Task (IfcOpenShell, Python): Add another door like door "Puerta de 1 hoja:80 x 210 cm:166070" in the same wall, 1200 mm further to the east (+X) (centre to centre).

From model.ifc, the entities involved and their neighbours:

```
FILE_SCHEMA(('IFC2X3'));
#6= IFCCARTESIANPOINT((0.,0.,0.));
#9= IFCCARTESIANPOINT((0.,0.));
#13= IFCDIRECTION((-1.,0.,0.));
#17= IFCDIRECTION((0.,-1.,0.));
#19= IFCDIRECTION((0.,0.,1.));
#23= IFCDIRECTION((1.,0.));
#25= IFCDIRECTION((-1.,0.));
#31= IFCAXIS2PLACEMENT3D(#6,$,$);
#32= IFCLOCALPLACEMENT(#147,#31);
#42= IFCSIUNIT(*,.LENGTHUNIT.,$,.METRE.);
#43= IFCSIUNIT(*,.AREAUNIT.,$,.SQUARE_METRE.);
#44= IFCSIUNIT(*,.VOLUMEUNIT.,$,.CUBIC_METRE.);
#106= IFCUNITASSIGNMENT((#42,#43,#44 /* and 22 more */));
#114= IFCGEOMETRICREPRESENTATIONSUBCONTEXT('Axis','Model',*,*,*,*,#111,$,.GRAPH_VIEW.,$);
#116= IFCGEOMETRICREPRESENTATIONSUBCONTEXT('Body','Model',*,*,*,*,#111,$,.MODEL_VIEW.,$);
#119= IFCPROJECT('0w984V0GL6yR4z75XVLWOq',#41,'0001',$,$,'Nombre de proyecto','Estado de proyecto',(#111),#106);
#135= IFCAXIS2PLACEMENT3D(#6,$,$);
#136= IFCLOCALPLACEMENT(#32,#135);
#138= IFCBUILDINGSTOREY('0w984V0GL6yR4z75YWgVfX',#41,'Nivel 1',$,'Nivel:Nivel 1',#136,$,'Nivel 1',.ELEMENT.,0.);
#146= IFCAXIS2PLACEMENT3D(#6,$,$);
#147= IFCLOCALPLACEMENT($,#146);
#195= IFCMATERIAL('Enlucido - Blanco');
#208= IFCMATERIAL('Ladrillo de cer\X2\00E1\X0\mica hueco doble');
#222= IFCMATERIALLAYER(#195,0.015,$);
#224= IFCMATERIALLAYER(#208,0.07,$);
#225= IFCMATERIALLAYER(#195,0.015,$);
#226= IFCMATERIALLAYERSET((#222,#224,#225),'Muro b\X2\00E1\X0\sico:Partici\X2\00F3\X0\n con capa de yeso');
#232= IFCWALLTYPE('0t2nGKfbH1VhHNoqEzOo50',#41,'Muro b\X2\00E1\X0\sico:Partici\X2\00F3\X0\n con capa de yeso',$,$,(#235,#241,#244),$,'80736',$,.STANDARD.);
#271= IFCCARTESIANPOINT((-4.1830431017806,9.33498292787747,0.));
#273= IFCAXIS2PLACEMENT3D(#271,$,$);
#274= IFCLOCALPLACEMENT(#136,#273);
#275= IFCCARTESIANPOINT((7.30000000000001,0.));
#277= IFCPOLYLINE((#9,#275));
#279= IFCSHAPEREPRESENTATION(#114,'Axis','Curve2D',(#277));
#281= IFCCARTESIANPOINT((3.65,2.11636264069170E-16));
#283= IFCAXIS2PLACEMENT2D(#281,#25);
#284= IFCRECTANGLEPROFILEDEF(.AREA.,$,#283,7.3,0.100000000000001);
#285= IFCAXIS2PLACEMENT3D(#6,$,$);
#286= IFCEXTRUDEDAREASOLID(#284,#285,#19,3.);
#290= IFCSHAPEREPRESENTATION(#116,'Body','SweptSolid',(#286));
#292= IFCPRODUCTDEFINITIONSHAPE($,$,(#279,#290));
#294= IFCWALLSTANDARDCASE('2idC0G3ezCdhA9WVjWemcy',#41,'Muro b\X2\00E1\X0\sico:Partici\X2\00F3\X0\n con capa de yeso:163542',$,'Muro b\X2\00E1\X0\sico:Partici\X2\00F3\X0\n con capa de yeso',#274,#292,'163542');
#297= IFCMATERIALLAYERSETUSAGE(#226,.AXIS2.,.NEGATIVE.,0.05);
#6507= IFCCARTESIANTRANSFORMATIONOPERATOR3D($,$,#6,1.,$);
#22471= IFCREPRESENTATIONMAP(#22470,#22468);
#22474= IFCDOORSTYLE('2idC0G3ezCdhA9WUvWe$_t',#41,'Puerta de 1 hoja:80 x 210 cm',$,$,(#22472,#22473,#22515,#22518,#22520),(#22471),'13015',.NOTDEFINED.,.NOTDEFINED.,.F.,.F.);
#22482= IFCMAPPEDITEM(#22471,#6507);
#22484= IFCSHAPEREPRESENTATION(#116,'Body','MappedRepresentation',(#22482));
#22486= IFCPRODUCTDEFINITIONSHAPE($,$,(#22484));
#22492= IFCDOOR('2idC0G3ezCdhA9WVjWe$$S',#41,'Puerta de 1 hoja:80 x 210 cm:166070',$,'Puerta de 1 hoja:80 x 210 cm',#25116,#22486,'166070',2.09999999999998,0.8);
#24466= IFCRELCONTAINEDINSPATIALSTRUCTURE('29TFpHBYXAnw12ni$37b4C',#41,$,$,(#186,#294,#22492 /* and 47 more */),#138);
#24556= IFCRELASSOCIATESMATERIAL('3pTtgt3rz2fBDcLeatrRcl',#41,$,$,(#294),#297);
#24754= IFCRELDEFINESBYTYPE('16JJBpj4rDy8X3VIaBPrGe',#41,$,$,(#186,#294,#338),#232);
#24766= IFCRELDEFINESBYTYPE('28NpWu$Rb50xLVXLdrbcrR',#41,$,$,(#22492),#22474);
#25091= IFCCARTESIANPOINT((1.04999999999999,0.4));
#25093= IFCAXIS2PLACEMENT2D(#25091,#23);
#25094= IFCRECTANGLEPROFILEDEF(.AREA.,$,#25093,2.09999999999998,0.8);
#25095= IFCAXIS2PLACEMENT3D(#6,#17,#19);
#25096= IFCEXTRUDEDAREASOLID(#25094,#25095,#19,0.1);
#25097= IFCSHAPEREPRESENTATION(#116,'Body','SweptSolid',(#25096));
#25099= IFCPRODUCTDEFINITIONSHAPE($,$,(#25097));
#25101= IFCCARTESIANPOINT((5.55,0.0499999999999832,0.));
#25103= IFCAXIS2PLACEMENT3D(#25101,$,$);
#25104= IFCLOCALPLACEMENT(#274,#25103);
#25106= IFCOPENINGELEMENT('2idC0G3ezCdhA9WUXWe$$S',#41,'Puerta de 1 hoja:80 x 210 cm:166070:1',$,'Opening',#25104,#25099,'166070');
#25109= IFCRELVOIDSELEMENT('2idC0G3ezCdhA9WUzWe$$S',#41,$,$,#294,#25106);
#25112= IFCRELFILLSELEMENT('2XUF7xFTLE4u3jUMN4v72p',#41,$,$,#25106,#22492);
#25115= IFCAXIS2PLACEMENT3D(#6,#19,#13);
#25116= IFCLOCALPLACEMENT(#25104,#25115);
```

```python
import ifcopenshell
import ifcopenshell.api.feature
import ifcopenshell.api.geometry
import ifcopenshell.api.root
import ifcopenshell.geom
import ifcopenshell.util.element
import ifcopenshell.util.placement
import ifcopenshell.util.shape
import ifcopenshell.util.unit

model = ifcopenshell.open("model.ifc")
unit_scale = ifcopenshell.util.unit.calculate_unit_scale(model)
settings = ifcopenshell.geom.settings()


def volume(element):
    """Net volume in cubic metres, openings subtracted."""
    shape = ifcopenshell.geom.create_shape(settings, element)
    return ifcopenshell.util.shape.get_volume(shape.geometry)


def reuse_history(source, copy):
    """copy_class also copies each property set's owner history, people and application; keep the originals."""
    for rel in copy.IsDefinedBy:
        if rel.is_a("IfcRelDefinesByProperties") and (history := rel.RelatingPropertyDefinition.OwnerHistory):
            rel.RelatingPropertyDefinition.OwnerHistory = source.OwnerHistory
            ifcopenshell.util.element.remove_deep2(model, history)


door = model.by_guid("2idC0G3ezCdhA9WVjWe$$S")
opening = door.FillsVoids[0].RelatingOpeningElement
wall = opening.VoidsElements[0].RelatingBuildingElement
before = volume(wall)
shift = ifcopenshell.util.placement.get_local_placement(wall.ObjectPlacement)[:3, 0] * 1.2 / unit_scale

# copy_class copies the void relationship, type, container and properties, but no geometry.
new_opening = ifcopenshell.api.root.copy_class(model, product=opening)
new_opening.Representation = ifcopenshell.util.element.copy_deep(
    model, opening.Representation, exclude=["IfcGeometricRepresentationContext", "IfcRepresentationMap"]
)
new_opening.Name = "Puerta de 1 hoja:80 x 210 cm"
new_opening.Tag = None
new_door = ifcopenshell.api.root.copy_class(model, product=door)
new_door.Representation = ifcopenshell.util.element.copy_deep(
    model, door.Representation, exclude=["IfcGeometricRepresentationContext", "IfcRepresentationMap"]
)
new_door.Name = "Puerta de 1 hoja:80 x 210 cm"
new_door.Tag = None
reuse_history(door, new_door)
fills = ifcopenshell.api.feature.add_filling(model, opening=new_opening, element=new_door)
fills.OwnerHistory = new_door.OwnerHistory  # required in IFC2X3

for old, new in ((opening, new_opening), (door, new_door)):
    matrix = ifcopenshell.util.placement.get_local_placement(old.ObjectPlacement)
    matrix[:3, 3] += shift
    ifcopenshell.api.geometry.edit_object_placement(model, product=new, matrix=matrix, is_si=False)

after = volume(wall)

print(f"wall volume {before:.3f} -> {after:.3f} m3")

model.write("model_rev.ifc")
```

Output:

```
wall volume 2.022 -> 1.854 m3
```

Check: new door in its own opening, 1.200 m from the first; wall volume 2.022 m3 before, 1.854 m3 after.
